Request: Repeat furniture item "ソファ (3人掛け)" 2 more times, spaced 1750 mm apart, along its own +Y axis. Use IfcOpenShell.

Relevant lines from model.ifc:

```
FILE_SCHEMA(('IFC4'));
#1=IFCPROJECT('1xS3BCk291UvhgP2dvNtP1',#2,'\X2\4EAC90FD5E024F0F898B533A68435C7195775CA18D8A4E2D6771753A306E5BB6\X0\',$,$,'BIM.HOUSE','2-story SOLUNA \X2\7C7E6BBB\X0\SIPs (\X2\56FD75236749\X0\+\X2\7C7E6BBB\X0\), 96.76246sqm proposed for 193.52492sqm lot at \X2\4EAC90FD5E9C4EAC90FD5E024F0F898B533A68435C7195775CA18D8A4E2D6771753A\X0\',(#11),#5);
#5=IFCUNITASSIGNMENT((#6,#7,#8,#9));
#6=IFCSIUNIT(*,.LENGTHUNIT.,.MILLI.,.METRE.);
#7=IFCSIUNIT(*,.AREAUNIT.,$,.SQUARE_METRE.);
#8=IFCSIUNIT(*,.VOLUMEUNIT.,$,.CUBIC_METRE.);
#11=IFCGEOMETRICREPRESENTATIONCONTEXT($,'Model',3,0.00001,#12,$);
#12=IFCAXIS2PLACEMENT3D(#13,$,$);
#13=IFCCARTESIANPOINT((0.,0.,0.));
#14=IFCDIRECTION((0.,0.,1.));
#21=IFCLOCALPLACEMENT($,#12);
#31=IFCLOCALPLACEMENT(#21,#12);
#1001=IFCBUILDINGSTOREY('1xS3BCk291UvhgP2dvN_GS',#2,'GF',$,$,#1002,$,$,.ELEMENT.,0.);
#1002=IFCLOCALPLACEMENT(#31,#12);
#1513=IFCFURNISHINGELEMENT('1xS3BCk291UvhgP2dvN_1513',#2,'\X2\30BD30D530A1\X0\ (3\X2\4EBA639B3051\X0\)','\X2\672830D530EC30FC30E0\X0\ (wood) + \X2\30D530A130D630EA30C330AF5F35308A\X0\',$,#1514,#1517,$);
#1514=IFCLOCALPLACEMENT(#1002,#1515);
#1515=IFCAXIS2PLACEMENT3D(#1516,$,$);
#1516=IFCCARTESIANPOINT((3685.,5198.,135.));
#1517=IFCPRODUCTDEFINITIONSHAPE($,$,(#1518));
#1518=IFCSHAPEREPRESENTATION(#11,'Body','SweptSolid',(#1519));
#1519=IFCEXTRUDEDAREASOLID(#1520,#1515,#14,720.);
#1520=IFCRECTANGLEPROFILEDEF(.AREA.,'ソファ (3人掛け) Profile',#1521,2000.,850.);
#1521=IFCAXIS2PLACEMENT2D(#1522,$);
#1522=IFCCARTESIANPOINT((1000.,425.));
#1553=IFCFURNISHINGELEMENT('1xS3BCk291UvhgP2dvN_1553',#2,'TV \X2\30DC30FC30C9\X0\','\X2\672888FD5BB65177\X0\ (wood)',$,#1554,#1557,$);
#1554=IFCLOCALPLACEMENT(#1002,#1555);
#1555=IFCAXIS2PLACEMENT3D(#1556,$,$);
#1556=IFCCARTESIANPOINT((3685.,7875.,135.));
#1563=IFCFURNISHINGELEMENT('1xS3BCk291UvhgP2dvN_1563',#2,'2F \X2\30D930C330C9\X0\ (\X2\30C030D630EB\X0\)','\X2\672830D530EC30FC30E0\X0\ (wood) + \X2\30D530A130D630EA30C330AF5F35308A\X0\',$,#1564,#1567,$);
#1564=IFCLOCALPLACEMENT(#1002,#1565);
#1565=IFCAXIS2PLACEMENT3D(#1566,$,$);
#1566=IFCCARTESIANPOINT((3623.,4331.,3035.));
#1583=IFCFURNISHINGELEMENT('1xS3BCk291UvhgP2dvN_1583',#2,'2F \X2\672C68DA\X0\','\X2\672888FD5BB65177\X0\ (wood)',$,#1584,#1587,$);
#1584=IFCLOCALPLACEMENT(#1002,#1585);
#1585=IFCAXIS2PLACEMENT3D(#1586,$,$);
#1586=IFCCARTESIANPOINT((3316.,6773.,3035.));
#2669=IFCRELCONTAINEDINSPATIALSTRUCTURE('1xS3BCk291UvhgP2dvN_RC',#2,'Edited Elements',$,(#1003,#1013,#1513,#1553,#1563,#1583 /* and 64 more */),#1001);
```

```python
import ifcopenshell
import ifcopenshell.api.geometry
import ifcopenshell.api.root
import ifcopenshell.util.element
import ifcopenshell.util.placement
import ifcopenshell.util.unit

model = ifcopenshell.open("model.ifc")
unit_scale = ifcopenshell.util.unit.calculate_unit_scale(model)


def reuse_history(source, copy):
    """copy_class also copies each property set's owner history, people and application; keep the originals."""
    for rel in copy.IsDefinedBy:
        if rel.is_a("IfcRelDefinesByProperties") and (history := rel.RelatingPropertyDefinition.OwnerHistory):
            rel.RelatingPropertyDefinition.OwnerHistory = source.OwnerHistory
            ifcopenshell.util.element.remove_deep2(model, history)


source = model.by_id(1513)
base = ifcopenshell.util.placement.get_local_placement(source.ObjectPlacement)
step = base[:3, 1] * 1.75 / unit_scale

for i in range(1, 3):
    copy = ifcopenshell.api.root.copy_class(model, product=source)
    copy.Representation = ifcopenshell.util.element.copy_deep(
        model, source.Representation, exclude=["IfcGeometricRepresentationContext", "IfcRepresentationMap"]
    )
    reuse_history(source, copy)
    matrix = base.copy()
    matrix[:3, 3] += i * step
    print("added at", matrix[:3, 3].round(3) + 0.0)
    ifcopenshell.api.geometry.edit_object_placement(model, product=copy, matrix=matrix, is_si=False)

model.write("model_edited.ifc")
```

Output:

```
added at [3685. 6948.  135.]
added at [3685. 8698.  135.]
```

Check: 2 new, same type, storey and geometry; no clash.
